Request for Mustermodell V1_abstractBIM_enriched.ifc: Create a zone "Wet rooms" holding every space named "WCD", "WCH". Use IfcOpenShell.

First a look at what the model holds.

```python
import ifcopenshell

model = ifcopenshell.open("Mustermodell V1_abstractBIM_enriched.ifc")
print(model.schema)
seen = {}
for space in model.by_type("IfcSpace"):
    seen[space.LongName] = seen.get(space.LongName, 0) + 1
for name, count in sorted(seen.items(), key=str):
    print(count, "x", name)
print("zones:", [z.Name for z in model.by_type("IfcZone")][:20])
```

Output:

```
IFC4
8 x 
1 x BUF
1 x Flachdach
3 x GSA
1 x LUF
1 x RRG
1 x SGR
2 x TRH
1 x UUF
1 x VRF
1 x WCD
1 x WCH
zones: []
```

```python
import ifcopenshell
import ifcopenshell.api.group
import ifcopenshell.api.root

model = ifcopenshell.open("Mustermodell V1_abstractBIM_enriched.ifc")

names = {"WCD", "WCH"}
spaces = [s for s in model.by_type("IfcSpace") if s.LongName in names]

zone = ifcopenshell.api.root.create_entity(model, ifc_class="IfcZone", name="Wet rooms")
ifcopenshell.api.group.assign_group(model, products=spaces, group=zone)
print(len(spaces), "spaces in", zone.Name)

model.write("Mustermodell V1_abstractBIM_enriched_rev.ifc")
```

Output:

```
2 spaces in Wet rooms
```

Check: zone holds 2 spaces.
